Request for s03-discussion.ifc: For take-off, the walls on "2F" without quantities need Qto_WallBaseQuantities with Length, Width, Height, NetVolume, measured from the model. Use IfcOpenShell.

First a look at what the model holds.

```python
import ifcopenshell
import ifcopenshell.util.element
import ifcopenshell.util.unit

model = ifcopenshell.open("s03-discussion.ifc")
print(model.schema)
for unit_type in ("LENGTHUNIT", "AREAUNIT", "VOLUMEUNIT"):
    print(unit_type, ifcopenshell.util.unit.calculate_unit_scale(model, unit_type))
storey = next(s for s in model.by_type("IfcBuildingStorey") if s.Name == "2F")
walls = [e for e in ifcopenshell.util.element.get_decomposition(storey) if e.is_a("IfcWall")]
for e in sorted(walls, key=lambda e: e.id()):
    print(e.id(), e.is_a(), e.Name, list(ifcopenshell.util.element.get_psets(e, qtos_only=True)), sep=" | ")
```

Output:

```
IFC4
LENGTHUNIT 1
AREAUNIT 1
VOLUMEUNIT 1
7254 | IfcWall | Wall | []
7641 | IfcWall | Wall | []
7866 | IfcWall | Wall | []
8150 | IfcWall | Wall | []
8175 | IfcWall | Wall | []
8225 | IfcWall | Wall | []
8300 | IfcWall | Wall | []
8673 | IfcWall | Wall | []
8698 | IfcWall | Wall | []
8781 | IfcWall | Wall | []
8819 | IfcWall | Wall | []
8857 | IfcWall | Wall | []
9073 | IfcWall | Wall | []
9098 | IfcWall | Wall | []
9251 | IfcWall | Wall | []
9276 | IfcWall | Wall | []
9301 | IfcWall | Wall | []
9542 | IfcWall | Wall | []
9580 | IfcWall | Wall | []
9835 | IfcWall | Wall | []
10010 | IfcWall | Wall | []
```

```python
import ifcopenshell
import ifcopenshell.api.pset
import ifcopenshell.geom
import ifcopenshell.util.element
import ifcopenshell.util.shape
import ifcopenshell.util.unit

model = ifcopenshell.open("s03-discussion.ifc")
unit_scale = ifcopenshell.util.unit.calculate_unit_scale(model)
volume_scale = ifcopenshell.util.unit.calculate_unit_scale(model, "VOLUMEUNIT")
settings = ifcopenshell.geom.settings()

storey = next(s for s in model.by_type("IfcBuildingStorey") if s.Name == "2F")
walls = [e for e in ifcopenshell.util.element.get_decomposition(storey) if e.is_a("IfcWall")]

for e in sorted(walls, key=lambda e: e.id()):
    if ifcopenshell.util.element.get_psets(e, qtos_only=True, should_inherit=False):
        continue
    # Geometry comes back in metres, in the element's own axes.
    shape = ifcopenshell.geom.create_shape(settings, e)
    values = {
        "Length": ifcopenshell.util.shape.get_x(shape.geometry) / unit_scale,
        "Width": ifcopenshell.util.shape.get_y(shape.geometry) / unit_scale,
        "Height": ifcopenshell.util.shape.get_z(shape.geometry) / unit_scale,
        "NetVolume": ifcopenshell.util.shape.get_volume(shape.geometry) / volume_scale,
    }
    qto = ifcopenshell.api.pset.add_qto(model, product=e, name="Qto_WallBaseQuantities")
    ifcopenshell.api.pset.edit_qto(model, qto=qto, properties=values)
    print(e.id(), {k: round(v, 3) for k, v in values.items()})

model.write("s03-discussion-out.ifc")
```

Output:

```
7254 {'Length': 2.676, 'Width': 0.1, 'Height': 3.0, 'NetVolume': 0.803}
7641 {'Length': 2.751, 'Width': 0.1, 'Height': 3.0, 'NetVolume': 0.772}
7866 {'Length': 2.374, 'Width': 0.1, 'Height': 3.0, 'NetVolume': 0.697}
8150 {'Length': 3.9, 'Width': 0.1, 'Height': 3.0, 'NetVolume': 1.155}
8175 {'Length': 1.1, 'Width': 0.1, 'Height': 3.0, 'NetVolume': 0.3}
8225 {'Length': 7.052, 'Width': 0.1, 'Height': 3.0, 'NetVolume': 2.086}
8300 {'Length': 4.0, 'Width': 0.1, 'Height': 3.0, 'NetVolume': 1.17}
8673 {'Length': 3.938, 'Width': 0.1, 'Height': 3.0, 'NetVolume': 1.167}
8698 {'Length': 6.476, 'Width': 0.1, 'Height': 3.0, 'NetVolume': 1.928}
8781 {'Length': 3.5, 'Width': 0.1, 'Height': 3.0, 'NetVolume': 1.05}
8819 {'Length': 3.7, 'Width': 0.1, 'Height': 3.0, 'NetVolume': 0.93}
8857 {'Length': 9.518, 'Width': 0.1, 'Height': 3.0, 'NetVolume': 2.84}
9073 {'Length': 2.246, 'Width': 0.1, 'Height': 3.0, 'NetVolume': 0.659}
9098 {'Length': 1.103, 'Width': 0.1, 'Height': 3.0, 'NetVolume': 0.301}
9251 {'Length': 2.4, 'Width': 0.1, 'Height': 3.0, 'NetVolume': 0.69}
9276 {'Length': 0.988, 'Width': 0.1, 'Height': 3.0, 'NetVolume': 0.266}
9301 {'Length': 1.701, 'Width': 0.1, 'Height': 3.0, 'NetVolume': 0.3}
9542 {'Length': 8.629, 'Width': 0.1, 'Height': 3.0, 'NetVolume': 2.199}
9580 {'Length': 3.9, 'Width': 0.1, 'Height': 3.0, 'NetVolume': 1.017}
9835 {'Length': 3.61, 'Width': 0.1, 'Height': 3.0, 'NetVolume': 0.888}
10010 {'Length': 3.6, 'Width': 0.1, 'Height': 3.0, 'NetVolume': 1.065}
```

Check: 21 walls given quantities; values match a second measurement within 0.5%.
